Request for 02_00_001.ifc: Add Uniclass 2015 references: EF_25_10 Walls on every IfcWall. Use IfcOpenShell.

First a look at what the model holds.

```python
import ifcopenshell

model = ifcopenshell.open("02_00_001.ifc")
print(model.schema)
print("classifications:", [c.Name for c in model.by_type("IfcClassification")])
for ifc_class in ("IfcDoor", "IfcRoof", "IfcStair", "IfcWall", "IfcWindow"):
    print(ifc_class, len(model.by_type(ifc_class)))
```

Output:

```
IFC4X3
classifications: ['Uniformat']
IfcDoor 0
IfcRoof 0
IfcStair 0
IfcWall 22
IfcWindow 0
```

```python
import ifcopenshell
import ifcopenshell.api.classification

model = ifcopenshell.open("02_00_001.ifc")

system = ifcopenshell.api.classification.add_classification(model, classification="Uniclass 2015")

codes = {
    "IfcWall": ("EF_25_10", "Walls"),
}
for ifc_class, (code, name) in codes.items():
    products = model.by_type(ifc_class)
    ifcopenshell.api.classification.add_reference(
        model, products=products, classification=system, identification=code, name=name
    )
    print(code, len(products))

model.write("02_00_001_v2.ifc")
```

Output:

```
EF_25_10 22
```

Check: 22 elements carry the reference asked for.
